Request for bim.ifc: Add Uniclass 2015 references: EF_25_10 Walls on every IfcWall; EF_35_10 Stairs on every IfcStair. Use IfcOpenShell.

First a look at what the model holds.

```python
import ifcopenshell

model = ifcopenshell.open("bim.ifc")
print(model.schema)
print("classifications:", [c.Name for c in model.by_type("IfcClassification")])
for ifc_class in ("IfcDoor", "IfcRoof", "IfcStair", "IfcWall", "IfcWindow"):
    print(ifc_class, len(model.by_type(ifc_class)))
```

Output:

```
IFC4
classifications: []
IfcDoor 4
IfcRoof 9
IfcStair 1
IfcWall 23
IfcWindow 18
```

```python
import ifcopenshell
import ifcopenshell.api.classification

model = ifcopenshell.open("bim.ifc")

system = ifcopenshell.api.classification.add_classification(model, classification="Uniclass 2015")

codes = {
    "IfcWall": ("EF_25_10", "Walls"),
    "IfcStair": ("EF_35_10", "Stairs"),
}
for ifc_class, (code, name) in codes.items():
    products = model.by_type(ifc_class)
    ifcopenshell.api.classification.add_reference(
        model, products=products, classification=system, identification=code, name=name
    )
    print(code, len(products))

model.write("bim_rev.ifc")
```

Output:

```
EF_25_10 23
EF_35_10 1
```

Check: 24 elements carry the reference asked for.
